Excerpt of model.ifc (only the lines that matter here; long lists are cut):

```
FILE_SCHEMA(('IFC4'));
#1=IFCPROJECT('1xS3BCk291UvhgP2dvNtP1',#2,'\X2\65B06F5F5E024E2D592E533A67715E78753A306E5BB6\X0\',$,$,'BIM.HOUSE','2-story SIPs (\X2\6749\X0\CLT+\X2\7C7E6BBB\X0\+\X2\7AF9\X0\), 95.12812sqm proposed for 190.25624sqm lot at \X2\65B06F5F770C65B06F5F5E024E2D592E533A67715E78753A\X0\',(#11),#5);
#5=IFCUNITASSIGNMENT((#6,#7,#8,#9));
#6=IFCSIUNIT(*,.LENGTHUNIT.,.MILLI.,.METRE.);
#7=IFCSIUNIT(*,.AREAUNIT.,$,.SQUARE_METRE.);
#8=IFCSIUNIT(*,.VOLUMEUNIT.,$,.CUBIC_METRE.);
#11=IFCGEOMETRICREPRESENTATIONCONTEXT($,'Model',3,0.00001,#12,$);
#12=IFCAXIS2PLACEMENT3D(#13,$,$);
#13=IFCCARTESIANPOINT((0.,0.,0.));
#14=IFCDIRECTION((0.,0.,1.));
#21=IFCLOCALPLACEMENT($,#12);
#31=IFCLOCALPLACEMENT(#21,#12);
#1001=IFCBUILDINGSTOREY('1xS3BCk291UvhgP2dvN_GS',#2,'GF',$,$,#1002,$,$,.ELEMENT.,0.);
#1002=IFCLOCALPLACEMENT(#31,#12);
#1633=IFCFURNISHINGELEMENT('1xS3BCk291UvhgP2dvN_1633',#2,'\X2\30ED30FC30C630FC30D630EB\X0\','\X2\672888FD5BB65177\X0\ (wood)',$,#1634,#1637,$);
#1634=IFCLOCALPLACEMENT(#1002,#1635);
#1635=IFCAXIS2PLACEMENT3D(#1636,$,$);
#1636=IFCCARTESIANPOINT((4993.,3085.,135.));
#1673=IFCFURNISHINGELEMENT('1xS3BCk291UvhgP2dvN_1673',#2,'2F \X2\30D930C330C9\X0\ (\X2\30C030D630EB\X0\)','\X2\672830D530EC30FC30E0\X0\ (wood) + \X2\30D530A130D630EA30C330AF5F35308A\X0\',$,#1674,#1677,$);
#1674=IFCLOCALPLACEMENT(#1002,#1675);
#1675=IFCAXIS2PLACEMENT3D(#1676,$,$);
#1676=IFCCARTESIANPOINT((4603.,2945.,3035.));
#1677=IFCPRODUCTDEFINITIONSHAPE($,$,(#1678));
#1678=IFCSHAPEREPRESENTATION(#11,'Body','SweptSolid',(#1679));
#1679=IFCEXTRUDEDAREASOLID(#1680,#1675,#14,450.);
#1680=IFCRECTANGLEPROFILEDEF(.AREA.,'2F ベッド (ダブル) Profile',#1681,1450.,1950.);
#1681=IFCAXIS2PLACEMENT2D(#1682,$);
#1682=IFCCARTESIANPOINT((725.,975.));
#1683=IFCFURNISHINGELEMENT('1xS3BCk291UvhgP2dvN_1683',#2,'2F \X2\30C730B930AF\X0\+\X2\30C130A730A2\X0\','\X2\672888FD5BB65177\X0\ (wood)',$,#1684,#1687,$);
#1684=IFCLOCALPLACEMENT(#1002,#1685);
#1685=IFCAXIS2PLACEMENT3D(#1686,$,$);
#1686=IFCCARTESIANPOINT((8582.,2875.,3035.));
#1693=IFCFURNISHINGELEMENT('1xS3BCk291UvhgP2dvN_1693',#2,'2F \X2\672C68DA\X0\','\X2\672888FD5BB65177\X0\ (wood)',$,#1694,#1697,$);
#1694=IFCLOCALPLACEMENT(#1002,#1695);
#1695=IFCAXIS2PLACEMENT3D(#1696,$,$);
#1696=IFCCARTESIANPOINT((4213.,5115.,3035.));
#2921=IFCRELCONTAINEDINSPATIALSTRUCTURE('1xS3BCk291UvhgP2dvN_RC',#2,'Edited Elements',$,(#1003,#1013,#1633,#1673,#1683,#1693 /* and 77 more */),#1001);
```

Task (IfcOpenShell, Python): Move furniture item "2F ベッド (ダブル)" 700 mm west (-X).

```python
import ifcopenshell
import ifcopenshell.api.geometry
import ifcopenshell.util.placement
import ifcopenshell.util.unit

model = ifcopenshell.open("model.ifc")
unit_scale = ifcopenshell.util.unit.calculate_unit_scale(model)

item = model.by_guid("1xS3BCk291UvhgP2dvN_1673")
matrix = ifcopenshell.util.placement.get_local_placement(item.ObjectPlacement)
matrix[0, 3] -= 0.7 / unit_scale
ifcopenshell.api.geometry.edit_object_placement(model, product=item, matrix=matrix, is_si=False)

print(ifcopenshell.util.placement.get_local_placement(item.ObjectPlacement).round(3) + 0.0)

model.write("model_edited.ifc")
```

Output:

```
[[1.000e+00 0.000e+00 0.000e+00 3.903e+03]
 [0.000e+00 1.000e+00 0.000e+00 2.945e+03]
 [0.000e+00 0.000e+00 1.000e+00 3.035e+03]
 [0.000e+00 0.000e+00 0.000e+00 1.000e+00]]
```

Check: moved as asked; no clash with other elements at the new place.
